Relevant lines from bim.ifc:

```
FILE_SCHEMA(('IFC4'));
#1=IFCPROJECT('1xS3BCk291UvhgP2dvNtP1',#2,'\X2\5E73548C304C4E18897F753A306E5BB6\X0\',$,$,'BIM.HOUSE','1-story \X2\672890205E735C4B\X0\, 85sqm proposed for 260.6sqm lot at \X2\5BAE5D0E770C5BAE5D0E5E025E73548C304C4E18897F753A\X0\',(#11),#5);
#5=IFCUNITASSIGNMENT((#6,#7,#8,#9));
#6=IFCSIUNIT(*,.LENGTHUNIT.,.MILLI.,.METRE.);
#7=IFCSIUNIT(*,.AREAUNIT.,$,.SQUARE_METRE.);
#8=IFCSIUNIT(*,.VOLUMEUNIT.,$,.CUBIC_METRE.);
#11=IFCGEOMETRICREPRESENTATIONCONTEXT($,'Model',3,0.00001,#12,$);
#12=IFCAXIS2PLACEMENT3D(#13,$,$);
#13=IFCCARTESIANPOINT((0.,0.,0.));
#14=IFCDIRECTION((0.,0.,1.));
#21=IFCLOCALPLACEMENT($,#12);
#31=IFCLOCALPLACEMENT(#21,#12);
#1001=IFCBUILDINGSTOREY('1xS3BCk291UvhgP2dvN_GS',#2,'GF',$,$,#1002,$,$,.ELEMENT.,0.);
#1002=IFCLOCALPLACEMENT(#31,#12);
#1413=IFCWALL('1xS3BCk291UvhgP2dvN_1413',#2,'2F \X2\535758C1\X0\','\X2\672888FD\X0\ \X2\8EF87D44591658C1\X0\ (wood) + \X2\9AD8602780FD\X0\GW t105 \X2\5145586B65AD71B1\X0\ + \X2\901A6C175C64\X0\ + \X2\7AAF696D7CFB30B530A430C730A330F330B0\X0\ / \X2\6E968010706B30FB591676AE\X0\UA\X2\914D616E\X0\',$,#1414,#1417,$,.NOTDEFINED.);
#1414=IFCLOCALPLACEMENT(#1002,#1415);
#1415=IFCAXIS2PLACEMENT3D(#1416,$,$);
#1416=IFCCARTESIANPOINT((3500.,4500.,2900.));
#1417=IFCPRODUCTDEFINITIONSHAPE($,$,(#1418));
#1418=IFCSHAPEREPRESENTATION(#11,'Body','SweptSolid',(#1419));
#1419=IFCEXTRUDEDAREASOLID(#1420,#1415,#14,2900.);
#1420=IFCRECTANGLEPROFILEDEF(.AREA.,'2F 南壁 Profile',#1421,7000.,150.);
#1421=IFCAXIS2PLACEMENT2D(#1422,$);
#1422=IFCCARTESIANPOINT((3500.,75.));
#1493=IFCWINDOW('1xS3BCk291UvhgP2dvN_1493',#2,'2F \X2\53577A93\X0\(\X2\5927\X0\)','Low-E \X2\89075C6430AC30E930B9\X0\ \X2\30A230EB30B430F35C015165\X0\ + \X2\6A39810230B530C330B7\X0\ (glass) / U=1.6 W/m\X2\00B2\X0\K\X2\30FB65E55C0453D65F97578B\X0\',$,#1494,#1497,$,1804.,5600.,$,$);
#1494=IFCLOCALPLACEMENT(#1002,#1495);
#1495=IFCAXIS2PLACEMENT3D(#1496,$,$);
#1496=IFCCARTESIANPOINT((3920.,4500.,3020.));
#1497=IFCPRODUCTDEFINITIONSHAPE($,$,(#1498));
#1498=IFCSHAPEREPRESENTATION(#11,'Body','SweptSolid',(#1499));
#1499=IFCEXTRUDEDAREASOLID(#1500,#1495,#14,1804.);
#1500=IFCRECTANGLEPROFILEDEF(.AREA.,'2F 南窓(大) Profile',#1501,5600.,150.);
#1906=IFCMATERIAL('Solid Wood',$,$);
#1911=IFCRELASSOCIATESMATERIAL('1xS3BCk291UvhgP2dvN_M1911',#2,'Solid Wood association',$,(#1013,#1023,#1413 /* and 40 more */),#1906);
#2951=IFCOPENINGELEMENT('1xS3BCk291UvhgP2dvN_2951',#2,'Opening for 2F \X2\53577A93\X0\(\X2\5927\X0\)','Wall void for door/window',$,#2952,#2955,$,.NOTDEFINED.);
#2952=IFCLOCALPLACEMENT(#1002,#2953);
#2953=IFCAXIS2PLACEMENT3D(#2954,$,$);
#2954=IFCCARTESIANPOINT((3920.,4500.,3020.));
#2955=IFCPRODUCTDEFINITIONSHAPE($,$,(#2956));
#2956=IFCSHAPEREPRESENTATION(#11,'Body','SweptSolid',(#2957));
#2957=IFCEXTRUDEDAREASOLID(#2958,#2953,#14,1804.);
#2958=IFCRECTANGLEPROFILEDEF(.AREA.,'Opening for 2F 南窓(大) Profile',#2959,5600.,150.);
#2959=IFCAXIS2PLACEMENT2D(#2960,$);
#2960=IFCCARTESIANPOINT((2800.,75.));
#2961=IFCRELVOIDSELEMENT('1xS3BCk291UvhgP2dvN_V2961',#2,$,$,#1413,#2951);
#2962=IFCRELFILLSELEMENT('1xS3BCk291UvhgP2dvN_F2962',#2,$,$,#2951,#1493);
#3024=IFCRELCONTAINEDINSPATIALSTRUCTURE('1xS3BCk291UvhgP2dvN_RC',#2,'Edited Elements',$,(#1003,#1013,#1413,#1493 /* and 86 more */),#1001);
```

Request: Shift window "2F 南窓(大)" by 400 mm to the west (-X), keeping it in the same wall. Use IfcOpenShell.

```python
import ifcopenshell
import ifcopenshell.api.geometry
import ifcopenshell.util.placement
import ifcopenshell.util.unit

model = ifcopenshell.open("bim.ifc")
unit_scale = ifcopenshell.util.unit.calculate_unit_scale(model)

window = model.by_guid("1xS3BCk291UvhgP2dvN_1493")
opening = window.FillsVoids[0].RelatingOpeningElement
wall = opening.VoidsElements[0].RelatingBuildingElement

wall_matrix = ifcopenshell.util.placement.get_local_placement(wall.ObjectPlacement)
shift = wall_matrix[:3, 0] * -0.4 / unit_scale
before = ifcopenshell.util.placement.get_local_placement(window.ObjectPlacement)[:3, 3].copy()

# The window is not placed relative to its opening, so move both.
for product in (opening, window):
    matrix = ifcopenshell.util.placement.get_local_placement(product.ObjectPlacement)
    matrix[:3, 3] += shift
    ifcopenshell.api.geometry.edit_object_placement(model, product=product, matrix=matrix, is_si=False)

after = ifcopenshell.util.placement.get_local_placement(window.ObjectPlacement)[:3, 3]
print("window moved by", (after - before).round(3) + 0.0)

model.write("bim_rev.ifc")
```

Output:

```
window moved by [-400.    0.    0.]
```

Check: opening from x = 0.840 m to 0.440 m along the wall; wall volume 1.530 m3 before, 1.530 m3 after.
